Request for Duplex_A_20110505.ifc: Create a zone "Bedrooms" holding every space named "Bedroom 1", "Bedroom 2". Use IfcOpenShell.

First a look at what the model holds.

```python
import ifcopenshell

model = ifcopenshell.open("Duplex_A_20110505.ifc")
print(model.schema)
seen = {}
for space in model.by_type("IfcSpace"):
    seen[space.LongName] = seen.get(space.LongName, 0) + 1
for name, count in sorted(seen.items(), key=str):
    print(count, "x", name)
print("zones:", [z.Name for z in model.by_type("IfcZone")][:20])
```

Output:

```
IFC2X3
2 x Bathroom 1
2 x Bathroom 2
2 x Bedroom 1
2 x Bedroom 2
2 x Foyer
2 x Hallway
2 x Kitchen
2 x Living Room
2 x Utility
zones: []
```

```python
import ifcopenshell
import ifcopenshell.api.group
import ifcopenshell.api.root

model = ifcopenshell.open("Duplex_A_20110505.ifc")

names = {"Bedroom 1", "Bedroom 2"}
spaces = [s for s in model.by_type("IfcSpace") if s.LongName in names]

zone = ifcopenshell.api.root.create_entity(model, ifc_class="IfcZone", name="Bedrooms")
ifcopenshell.api.group.assign_group(model, products=spaces, group=zone)
print(len(spaces), "spaces in", zone.Name)

model.write("Duplex_A_20110505_v2.ifc")
```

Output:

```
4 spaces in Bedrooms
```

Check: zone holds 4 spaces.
